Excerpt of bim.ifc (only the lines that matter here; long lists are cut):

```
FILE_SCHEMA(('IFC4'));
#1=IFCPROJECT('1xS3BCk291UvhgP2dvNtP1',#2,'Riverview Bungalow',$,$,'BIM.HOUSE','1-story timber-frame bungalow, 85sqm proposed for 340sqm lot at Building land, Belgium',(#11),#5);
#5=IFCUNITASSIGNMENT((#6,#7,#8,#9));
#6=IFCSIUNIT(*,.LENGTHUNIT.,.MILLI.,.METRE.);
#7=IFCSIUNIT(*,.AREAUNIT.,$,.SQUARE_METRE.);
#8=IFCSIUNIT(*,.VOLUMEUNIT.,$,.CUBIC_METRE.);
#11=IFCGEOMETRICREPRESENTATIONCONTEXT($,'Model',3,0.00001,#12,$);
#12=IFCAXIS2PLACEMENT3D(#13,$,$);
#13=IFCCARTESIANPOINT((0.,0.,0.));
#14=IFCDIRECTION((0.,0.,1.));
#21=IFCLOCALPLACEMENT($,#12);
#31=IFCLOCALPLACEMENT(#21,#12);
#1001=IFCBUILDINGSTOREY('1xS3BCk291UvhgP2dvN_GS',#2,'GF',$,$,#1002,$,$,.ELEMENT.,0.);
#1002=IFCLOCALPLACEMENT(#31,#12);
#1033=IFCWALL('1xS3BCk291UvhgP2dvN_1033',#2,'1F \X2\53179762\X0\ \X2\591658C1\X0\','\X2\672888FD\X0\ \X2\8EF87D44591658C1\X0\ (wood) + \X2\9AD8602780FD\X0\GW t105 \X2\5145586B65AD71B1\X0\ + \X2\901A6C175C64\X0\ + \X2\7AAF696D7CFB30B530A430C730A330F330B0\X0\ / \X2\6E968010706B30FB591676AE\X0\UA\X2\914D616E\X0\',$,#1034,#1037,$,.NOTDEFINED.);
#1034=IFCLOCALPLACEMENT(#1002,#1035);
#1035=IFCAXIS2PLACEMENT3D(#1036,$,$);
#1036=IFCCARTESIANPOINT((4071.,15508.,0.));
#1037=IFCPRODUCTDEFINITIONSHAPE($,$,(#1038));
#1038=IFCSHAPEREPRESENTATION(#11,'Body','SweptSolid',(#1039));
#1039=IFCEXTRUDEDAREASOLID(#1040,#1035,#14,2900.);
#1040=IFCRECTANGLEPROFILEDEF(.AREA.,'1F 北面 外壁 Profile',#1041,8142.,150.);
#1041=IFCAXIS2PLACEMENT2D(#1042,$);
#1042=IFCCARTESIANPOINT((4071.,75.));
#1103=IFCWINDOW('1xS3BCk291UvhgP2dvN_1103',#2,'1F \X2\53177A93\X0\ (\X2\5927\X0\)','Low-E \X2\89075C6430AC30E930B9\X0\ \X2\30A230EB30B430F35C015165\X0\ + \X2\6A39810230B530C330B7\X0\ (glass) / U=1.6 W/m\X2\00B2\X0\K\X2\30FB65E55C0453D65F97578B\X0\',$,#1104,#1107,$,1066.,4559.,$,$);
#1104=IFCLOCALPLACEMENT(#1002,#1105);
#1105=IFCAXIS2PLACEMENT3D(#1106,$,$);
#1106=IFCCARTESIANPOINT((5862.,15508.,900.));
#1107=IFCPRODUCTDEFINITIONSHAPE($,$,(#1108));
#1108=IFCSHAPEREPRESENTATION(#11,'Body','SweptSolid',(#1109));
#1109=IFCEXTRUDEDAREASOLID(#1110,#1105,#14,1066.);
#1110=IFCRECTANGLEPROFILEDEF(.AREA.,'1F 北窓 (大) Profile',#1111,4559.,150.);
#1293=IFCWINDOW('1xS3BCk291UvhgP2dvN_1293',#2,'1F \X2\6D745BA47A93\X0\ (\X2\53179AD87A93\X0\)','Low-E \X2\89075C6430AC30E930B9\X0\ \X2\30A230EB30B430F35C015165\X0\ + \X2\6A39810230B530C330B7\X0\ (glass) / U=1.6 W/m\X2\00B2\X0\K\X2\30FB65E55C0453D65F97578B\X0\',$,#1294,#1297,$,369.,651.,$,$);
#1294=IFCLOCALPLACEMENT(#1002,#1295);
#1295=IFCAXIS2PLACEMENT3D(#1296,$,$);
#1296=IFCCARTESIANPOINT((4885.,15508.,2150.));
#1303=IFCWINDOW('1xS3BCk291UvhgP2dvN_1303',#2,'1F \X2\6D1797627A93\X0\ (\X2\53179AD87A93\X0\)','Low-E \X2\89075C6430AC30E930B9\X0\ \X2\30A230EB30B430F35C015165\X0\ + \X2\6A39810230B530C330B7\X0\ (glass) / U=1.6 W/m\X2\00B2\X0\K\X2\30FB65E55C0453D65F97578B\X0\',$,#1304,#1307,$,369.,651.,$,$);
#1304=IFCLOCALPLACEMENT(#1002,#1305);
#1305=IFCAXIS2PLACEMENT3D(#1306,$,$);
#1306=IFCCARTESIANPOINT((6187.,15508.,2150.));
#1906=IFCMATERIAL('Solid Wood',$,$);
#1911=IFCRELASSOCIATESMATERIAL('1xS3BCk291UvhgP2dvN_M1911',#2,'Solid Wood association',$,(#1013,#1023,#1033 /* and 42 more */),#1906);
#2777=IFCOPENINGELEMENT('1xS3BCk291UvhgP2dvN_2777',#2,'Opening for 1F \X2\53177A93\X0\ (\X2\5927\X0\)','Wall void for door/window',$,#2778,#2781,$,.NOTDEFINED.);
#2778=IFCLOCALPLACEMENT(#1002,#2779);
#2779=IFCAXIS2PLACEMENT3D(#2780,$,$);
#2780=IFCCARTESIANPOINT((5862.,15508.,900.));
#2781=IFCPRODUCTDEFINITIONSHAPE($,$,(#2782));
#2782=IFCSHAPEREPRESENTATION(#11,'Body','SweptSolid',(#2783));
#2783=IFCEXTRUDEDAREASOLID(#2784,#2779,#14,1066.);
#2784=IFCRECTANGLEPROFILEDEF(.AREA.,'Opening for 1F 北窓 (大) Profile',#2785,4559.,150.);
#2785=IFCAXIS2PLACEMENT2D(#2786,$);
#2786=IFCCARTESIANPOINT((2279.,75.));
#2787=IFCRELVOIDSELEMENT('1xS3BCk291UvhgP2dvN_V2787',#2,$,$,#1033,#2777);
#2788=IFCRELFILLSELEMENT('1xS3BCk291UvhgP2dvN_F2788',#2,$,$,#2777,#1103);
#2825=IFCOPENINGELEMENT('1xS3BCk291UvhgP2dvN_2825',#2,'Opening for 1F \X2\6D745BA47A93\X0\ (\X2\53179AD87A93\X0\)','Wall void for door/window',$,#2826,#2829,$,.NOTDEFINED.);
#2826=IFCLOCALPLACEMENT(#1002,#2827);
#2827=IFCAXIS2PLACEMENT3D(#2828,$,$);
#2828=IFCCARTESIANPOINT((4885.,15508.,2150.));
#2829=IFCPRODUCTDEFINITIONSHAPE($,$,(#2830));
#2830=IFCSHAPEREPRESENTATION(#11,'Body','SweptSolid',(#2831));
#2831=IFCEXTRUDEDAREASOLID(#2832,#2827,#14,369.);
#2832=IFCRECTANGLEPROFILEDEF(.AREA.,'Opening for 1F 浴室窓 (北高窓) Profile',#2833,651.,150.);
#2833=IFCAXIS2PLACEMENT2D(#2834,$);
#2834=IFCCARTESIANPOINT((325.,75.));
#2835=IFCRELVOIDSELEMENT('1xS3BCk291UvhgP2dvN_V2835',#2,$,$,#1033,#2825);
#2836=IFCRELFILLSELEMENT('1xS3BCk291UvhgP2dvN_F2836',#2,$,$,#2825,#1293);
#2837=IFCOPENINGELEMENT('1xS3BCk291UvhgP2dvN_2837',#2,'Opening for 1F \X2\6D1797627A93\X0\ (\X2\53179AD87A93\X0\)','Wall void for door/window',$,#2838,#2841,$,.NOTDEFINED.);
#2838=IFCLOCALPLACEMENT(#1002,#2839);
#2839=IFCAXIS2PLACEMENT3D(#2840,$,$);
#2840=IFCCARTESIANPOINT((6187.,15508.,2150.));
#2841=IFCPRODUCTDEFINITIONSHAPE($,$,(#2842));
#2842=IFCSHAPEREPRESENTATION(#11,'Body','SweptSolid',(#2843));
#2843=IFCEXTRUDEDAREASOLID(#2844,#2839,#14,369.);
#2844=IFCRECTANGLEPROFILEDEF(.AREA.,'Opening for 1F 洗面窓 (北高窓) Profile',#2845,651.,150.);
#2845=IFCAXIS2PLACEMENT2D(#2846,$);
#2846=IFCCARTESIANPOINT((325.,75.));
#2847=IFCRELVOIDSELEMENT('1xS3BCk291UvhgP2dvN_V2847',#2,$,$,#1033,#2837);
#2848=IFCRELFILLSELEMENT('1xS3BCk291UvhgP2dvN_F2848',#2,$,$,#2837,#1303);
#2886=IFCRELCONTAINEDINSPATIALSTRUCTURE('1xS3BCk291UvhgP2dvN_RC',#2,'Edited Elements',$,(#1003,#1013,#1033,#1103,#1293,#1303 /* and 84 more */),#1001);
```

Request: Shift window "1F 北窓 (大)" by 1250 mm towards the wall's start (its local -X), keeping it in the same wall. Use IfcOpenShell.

```python
import ifcopenshell
import ifcopenshell.api.geometry
import ifcopenshell.util.placement
import ifcopenshell.util.unit

model = ifcopenshell.open("bim.ifc")
unit_scale = ifcopenshell.util.unit.calculate_unit_scale(model)

window = model.by_guid("1xS3BCk291UvhgP2dvN_1103")
opening = window.FillsVoids[0].RelatingOpeningElement
wall = opening.VoidsElements[0].RelatingBuildingElement

wall_matrix = ifcopenshell.util.placement.get_local_placement(wall.ObjectPlacement)
shift = wall_matrix[:3, 0] * -1.25 / unit_scale
before = ifcopenshell.util.placement.get_local_placement(window.ObjectPlacement)[:3, 3].copy()

# The window is not placed relative to its opening, so move both.
for product in (opening, window):
    matrix = ifcopenshell.util.placement.get_local_placement(product.ObjectPlacement)
    matrix[:3, 3] += shift
    ifcopenshell.api.geometry.edit_object_placement(model, product=product, matrix=matrix, is_si=False)

after = ifcopenshell.util.placement.get_local_placement(window.ObjectPlacement)[:3, 3]
print("window moved by", (after - before).round(3) + 0.0)

model.write("bim-out.ifc")
```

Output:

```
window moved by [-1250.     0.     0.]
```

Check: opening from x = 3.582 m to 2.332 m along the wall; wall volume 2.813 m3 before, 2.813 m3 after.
